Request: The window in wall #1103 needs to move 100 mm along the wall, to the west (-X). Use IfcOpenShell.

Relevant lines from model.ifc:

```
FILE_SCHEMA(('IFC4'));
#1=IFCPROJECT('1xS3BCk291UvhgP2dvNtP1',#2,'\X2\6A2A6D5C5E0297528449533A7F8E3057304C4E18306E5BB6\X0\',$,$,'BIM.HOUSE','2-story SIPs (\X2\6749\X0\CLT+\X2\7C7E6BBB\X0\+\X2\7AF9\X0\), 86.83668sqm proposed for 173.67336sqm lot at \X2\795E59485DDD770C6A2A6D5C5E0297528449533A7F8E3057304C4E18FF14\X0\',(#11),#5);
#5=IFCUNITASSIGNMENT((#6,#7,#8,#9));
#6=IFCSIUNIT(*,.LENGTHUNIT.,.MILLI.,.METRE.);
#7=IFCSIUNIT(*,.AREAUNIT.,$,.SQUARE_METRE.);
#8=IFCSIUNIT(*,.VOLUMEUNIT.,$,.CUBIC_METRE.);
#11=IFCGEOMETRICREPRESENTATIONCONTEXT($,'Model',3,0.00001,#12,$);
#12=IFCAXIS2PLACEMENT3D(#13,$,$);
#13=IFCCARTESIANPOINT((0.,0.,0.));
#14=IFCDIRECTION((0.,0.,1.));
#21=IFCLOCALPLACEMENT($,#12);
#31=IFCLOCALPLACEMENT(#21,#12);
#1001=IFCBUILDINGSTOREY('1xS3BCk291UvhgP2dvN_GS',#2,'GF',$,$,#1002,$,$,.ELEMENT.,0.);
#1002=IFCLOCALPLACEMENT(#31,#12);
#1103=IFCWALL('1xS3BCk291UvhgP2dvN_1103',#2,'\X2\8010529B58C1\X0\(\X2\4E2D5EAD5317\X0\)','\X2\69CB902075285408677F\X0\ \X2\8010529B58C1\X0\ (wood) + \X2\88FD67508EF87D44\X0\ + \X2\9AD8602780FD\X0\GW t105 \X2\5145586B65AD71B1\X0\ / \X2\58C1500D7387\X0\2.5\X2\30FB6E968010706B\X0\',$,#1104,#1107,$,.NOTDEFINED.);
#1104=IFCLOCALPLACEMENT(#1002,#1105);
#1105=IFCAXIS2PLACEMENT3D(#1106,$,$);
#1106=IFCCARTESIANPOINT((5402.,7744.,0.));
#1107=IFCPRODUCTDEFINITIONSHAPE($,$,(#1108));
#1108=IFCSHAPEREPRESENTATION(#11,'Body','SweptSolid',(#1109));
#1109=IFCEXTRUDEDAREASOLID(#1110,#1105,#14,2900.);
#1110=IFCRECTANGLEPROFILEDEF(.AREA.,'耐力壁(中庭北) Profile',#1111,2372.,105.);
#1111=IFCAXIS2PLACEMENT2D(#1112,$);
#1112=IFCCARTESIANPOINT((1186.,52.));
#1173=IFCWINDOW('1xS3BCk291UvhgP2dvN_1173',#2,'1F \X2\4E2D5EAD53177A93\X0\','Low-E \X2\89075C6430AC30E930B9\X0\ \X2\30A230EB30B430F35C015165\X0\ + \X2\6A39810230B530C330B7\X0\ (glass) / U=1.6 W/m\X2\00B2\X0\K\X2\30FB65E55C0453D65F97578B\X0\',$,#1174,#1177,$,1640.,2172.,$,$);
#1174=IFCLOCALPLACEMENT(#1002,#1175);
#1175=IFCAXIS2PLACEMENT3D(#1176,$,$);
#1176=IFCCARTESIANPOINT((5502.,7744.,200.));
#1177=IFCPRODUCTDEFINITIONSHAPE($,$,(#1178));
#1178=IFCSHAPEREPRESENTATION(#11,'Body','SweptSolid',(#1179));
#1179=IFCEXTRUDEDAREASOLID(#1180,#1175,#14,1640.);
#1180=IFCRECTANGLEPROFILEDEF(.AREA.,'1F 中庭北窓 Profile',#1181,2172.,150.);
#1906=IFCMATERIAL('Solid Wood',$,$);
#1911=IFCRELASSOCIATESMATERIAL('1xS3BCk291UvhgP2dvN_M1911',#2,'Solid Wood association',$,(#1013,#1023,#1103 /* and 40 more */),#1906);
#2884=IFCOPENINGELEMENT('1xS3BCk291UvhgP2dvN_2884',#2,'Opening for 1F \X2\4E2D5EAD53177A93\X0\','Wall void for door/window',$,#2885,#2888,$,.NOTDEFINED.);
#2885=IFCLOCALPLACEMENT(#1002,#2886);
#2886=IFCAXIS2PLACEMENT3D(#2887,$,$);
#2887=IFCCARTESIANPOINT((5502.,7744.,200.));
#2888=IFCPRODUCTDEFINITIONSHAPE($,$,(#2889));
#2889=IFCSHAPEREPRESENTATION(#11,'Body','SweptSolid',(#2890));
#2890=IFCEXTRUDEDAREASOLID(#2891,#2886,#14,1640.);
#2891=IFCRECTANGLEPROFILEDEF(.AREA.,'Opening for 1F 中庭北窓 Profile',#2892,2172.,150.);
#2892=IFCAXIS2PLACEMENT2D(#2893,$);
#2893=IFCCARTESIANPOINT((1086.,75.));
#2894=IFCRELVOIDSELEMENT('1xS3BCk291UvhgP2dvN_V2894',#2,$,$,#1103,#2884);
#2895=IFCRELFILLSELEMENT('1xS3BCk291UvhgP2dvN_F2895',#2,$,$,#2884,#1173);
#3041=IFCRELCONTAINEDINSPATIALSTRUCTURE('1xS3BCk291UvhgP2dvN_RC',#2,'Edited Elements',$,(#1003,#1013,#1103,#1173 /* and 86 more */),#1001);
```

```python
import ifcopenshell
import ifcopenshell.api.geometry
import ifcopenshell.util.placement
import ifcopenshell.util.unit

model = ifcopenshell.open("model.ifc")
unit_scale = ifcopenshell.util.unit.calculate_unit_scale(model)

window = model.by_guid("1xS3BCk291UvhgP2dvN_1173")
opening = window.FillsVoids[0].RelatingOpeningElement
wall = opening.VoidsElements[0].RelatingBuildingElement

wall_matrix = ifcopenshell.util.placement.get_local_placement(wall.ObjectPlacement)
shift = wall_matrix[:3, 0] * -0.1 / unit_scale
before = ifcopenshell.util.placement.get_local_placement(window.ObjectPlacement)[:3, 3].copy()

# The window is not placed relative to its opening, so move both.
for product in (opening, window):
    matrix = ifcopenshell.util.placement.get_local_placement(product.ObjectPlacement)
    matrix[:3, 3] += shift
    ifcopenshell.api.geometry.edit_object_placement(model, product=product, matrix=matrix, is_si=False)

after = ifcopenshell.util.placement.get_local_placement(window.ObjectPlacement)[:3, 3]
print("window moved by", (after - before).round(3) + 0.0)

model.write("model_v2.ifc")
```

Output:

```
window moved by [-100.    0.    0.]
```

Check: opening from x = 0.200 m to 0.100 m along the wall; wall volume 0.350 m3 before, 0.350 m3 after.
